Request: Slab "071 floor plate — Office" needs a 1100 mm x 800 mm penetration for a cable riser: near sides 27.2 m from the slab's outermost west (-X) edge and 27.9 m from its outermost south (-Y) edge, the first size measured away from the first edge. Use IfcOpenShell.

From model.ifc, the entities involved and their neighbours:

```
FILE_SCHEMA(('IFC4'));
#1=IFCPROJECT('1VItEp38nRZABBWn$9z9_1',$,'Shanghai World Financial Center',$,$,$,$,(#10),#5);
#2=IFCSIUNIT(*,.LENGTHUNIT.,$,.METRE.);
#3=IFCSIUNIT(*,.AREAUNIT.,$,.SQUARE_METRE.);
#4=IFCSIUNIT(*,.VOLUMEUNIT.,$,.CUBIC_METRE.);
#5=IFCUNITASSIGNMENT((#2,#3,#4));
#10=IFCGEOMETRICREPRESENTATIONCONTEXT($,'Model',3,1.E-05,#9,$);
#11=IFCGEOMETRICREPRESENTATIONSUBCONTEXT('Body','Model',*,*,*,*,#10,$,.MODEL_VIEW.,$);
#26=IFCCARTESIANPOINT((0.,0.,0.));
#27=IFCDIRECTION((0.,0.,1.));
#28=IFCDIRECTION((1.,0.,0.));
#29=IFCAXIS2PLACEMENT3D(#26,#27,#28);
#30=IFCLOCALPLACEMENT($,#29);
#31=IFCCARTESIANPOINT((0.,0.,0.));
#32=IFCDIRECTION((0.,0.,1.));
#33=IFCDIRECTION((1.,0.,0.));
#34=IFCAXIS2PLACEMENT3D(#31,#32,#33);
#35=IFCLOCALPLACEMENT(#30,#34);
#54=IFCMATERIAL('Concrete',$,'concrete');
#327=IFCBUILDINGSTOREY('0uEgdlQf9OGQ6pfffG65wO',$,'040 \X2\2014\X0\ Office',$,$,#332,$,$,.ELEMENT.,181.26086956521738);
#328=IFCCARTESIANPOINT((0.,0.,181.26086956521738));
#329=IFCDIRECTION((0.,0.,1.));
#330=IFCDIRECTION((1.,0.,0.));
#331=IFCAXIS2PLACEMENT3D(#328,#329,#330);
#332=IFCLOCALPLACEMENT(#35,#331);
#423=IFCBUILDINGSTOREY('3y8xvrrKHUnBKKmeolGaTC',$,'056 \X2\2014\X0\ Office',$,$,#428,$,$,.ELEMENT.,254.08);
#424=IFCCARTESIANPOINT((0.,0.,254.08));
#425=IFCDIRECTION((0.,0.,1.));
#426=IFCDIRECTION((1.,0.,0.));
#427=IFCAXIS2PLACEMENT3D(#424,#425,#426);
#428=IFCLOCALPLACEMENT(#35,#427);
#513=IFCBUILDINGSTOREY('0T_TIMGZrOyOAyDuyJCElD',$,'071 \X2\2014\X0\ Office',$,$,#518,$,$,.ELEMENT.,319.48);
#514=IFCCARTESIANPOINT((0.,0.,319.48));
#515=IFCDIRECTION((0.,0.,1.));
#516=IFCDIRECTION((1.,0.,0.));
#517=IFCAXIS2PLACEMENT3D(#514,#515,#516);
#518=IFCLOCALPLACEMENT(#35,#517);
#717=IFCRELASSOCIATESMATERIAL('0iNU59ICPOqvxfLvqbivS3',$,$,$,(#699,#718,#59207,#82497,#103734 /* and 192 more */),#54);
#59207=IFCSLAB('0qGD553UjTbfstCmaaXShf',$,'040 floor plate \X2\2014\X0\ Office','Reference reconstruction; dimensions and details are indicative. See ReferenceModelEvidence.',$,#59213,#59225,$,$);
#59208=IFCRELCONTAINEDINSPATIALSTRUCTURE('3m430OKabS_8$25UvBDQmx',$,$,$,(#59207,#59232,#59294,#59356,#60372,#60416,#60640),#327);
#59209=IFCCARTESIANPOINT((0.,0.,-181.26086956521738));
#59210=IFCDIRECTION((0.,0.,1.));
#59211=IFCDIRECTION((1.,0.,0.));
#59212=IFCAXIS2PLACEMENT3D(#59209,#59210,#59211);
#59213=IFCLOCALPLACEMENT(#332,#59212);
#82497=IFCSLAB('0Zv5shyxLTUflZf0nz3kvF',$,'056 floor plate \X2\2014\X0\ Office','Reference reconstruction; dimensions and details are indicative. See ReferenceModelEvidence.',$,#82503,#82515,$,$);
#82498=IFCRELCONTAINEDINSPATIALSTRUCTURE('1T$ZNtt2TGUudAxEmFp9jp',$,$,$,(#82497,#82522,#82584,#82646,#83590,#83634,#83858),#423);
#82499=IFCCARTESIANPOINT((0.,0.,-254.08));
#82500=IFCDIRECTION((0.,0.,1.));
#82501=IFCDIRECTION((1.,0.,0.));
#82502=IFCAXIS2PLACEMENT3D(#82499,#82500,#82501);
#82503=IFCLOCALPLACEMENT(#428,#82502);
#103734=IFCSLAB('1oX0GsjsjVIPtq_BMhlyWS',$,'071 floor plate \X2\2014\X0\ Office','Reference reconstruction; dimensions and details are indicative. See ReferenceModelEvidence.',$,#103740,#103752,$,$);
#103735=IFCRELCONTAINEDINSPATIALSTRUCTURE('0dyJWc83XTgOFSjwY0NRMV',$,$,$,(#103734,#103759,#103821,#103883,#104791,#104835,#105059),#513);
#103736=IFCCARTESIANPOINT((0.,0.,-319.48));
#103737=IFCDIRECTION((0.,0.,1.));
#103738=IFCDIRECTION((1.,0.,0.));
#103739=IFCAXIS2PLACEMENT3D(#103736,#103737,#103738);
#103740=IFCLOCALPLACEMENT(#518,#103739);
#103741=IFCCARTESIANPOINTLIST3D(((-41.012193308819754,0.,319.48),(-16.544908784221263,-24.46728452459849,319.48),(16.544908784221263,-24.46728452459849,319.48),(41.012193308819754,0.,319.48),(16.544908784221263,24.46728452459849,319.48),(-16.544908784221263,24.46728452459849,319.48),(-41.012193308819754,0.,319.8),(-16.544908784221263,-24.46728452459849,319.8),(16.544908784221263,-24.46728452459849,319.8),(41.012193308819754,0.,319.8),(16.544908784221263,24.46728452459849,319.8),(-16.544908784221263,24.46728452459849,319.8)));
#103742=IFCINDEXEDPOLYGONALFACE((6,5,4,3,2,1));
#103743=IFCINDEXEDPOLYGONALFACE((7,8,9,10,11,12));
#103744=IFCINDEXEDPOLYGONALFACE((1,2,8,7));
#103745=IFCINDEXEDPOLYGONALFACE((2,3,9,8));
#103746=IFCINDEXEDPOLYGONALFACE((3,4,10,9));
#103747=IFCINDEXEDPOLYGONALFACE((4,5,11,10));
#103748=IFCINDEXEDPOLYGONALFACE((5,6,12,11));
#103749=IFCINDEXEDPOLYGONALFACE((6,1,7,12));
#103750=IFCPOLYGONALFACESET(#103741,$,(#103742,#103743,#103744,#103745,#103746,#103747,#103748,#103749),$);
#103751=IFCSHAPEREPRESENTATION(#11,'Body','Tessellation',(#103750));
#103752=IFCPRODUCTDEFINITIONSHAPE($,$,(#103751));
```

```python
import numpy as np
import ifcopenshell
import ifcopenshell.api.feature
import ifcopenshell.api.geometry
import ifcopenshell.api.root
import ifcopenshell.geom
import ifcopenshell.util.placement
import ifcopenshell.util.representation
import ifcopenshell.util.shape
import ifcopenshell.util.unit

model = ifcopenshell.open("model.ifc")
unit_scale = ifcopenshell.util.unit.calculate_unit_scale(model)
settings = ifcopenshell.geom.settings()


def volume(element):
    """Net volume in cubic metres, openings subtracted."""
    shape = ifcopenshell.geom.create_shape(settings, element)
    return ifcopenshell.util.shape.get_volume(shape.geometry)


slab = model.by_guid("1oX0GsjsjVIPtq_BMhlyWS")
before = volume(slab)

# Extent in the slab's own axes, in metres. The edges named are its -X and -Y sides.
slab_shape = ifcopenshell.geom.create_shape(settings, slab)
vertices = ifcopenshell.util.shape.get_vertices(slab_shape.geometry)
x_min, y_min, bottom = vertices.min(axis=0)
top = vertices[:, 2].max()

opening = ifcopenshell.api.root.create_entity(model, ifc_class="IfcOpeningElement", name="Cable riser opening", predefined_type="OPENING")
context = ifcopenshell.util.representation.get_context(model, "Model", "Body", "MODEL_VIEW")
width, depth = 1.1, 0.8
outline = [(0.0, 0.0), (width, 0.0), (width, depth), (0.0, depth), (0.0, 0.0)]
# Overshoot both faces by 50 mm so the cut is clean.
shape = ifcopenshell.api.geometry.add_slab_representation(
    model, context=context, depth=top - bottom + 0.1, polyline=outline
)
ifcopenshell.api.geometry.assign_representation(model, product=opening, representation=shape)

matrix = ifcopenshell.util.placement.get_local_placement(slab.ObjectPlacement)
matrix[:, 3] = matrix @ np.append(np.array([x_min + 27.2, y_min + 27.9, bottom - 0.05]) / unit_scale, 1.0)
ifcopenshell.api.geometry.edit_object_placement(model, product=opening, matrix=matrix, is_si=False)
ifcopenshell.api.feature.add_feature(model, feature=opening, element=slab)

after = volume(slab)

print(f"slab volume {before:.3f} -> {after:.3f} m3")

model.write("model_updated.ifc")
```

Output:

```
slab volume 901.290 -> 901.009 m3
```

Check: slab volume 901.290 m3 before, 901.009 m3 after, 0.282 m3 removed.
